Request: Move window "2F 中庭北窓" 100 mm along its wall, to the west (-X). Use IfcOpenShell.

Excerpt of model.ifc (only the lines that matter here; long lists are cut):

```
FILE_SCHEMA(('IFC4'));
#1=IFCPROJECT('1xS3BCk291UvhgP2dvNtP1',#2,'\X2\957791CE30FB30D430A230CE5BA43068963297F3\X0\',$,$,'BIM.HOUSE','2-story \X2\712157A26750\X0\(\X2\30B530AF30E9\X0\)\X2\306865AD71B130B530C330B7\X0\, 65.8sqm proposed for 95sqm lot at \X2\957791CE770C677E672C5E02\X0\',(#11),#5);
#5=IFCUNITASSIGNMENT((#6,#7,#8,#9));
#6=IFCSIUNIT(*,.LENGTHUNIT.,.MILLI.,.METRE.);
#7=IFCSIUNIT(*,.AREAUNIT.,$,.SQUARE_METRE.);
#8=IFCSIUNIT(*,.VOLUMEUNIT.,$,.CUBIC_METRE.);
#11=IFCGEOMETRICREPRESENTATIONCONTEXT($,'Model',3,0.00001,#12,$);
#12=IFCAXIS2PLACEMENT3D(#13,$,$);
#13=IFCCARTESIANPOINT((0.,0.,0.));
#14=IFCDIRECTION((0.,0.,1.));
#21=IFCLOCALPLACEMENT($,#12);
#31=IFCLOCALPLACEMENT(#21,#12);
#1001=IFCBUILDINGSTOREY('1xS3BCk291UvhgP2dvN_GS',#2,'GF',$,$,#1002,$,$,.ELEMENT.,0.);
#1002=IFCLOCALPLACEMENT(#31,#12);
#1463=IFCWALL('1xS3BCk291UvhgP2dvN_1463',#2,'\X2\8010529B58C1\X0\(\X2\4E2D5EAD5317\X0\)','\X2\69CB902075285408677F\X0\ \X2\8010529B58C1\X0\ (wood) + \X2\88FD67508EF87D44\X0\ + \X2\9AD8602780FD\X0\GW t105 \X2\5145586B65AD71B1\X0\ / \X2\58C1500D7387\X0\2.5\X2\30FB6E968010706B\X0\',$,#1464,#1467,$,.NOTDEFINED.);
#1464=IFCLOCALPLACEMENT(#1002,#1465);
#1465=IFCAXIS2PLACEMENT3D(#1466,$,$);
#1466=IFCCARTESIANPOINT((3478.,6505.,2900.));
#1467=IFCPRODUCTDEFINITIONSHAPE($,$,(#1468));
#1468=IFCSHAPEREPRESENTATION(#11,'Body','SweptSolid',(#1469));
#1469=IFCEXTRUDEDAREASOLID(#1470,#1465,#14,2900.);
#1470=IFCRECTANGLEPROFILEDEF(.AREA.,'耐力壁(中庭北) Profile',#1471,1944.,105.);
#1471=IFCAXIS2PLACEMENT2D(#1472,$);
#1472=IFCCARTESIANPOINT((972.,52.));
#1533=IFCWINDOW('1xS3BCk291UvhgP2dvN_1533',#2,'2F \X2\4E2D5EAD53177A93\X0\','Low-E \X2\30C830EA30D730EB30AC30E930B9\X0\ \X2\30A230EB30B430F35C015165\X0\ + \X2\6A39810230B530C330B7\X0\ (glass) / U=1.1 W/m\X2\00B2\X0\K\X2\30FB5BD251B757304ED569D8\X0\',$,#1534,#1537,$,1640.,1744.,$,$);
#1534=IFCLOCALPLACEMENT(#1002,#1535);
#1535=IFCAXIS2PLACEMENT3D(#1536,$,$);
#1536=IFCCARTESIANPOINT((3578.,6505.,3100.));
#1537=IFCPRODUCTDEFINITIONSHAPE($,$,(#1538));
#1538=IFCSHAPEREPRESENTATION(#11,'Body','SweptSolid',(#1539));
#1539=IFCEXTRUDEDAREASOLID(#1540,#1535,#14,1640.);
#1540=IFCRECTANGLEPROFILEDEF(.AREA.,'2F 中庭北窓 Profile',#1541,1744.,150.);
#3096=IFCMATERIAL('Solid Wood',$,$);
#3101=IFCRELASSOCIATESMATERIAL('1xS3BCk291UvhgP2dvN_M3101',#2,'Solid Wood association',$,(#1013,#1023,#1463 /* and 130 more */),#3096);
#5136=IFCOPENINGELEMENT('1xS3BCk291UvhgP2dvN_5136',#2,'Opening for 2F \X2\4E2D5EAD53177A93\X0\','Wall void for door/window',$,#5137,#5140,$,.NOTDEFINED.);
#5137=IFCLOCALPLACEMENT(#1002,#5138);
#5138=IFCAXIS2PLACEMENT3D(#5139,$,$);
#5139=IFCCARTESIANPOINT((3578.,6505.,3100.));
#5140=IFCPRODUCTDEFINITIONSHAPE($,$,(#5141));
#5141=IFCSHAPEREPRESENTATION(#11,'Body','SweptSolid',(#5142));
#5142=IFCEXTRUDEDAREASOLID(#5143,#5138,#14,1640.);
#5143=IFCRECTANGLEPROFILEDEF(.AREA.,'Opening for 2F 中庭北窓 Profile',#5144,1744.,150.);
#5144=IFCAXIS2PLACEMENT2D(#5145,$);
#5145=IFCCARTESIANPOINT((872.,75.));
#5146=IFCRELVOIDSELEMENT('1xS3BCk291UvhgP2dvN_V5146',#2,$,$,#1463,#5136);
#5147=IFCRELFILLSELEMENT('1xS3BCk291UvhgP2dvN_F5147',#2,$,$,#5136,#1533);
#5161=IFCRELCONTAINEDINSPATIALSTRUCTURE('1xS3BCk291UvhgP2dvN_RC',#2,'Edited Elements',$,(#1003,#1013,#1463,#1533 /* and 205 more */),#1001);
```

```python
import ifcopenshell
import ifcopenshell.api.geometry
import ifcopenshell.util.placement
import ifcopenshell.util.unit

model = ifcopenshell.open("model.ifc")
unit_scale = ifcopenshell.util.unit.calculate_unit_scale(model)

window = model.by_guid("1xS3BCk291UvhgP2dvN_1533")
opening = window.FillsVoids[0].RelatingOpeningElement
wall = opening.VoidsElements[0].RelatingBuildingElement

wall_matrix = ifcopenshell.util.placement.get_local_placement(wall.ObjectPlacement)
shift = wall_matrix[:3, 0] * -0.1 / unit_scale
before = ifcopenshell.util.placement.get_local_placement(window.ObjectPlacement)[:3, 3].copy()

# The window is not placed relative to its opening, so move both.
for product in (opening, window):
    matrix = ifcopenshell.util.placement.get_local_placement(product.ObjectPlacement)
    matrix[:3, 3] += shift
    ifcopenshell.api.geometry.edit_object_placement(model, product=product, matrix=matrix, is_si=False)

after = ifcopenshell.util.placement.get_local_placement(window.ObjectPlacement)[:3, 3]
print("window moved by", (after - before).round(3) + 0.0)

model.write("model-out.ifc")
```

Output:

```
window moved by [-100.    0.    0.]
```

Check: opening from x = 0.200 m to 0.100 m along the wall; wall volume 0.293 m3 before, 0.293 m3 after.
